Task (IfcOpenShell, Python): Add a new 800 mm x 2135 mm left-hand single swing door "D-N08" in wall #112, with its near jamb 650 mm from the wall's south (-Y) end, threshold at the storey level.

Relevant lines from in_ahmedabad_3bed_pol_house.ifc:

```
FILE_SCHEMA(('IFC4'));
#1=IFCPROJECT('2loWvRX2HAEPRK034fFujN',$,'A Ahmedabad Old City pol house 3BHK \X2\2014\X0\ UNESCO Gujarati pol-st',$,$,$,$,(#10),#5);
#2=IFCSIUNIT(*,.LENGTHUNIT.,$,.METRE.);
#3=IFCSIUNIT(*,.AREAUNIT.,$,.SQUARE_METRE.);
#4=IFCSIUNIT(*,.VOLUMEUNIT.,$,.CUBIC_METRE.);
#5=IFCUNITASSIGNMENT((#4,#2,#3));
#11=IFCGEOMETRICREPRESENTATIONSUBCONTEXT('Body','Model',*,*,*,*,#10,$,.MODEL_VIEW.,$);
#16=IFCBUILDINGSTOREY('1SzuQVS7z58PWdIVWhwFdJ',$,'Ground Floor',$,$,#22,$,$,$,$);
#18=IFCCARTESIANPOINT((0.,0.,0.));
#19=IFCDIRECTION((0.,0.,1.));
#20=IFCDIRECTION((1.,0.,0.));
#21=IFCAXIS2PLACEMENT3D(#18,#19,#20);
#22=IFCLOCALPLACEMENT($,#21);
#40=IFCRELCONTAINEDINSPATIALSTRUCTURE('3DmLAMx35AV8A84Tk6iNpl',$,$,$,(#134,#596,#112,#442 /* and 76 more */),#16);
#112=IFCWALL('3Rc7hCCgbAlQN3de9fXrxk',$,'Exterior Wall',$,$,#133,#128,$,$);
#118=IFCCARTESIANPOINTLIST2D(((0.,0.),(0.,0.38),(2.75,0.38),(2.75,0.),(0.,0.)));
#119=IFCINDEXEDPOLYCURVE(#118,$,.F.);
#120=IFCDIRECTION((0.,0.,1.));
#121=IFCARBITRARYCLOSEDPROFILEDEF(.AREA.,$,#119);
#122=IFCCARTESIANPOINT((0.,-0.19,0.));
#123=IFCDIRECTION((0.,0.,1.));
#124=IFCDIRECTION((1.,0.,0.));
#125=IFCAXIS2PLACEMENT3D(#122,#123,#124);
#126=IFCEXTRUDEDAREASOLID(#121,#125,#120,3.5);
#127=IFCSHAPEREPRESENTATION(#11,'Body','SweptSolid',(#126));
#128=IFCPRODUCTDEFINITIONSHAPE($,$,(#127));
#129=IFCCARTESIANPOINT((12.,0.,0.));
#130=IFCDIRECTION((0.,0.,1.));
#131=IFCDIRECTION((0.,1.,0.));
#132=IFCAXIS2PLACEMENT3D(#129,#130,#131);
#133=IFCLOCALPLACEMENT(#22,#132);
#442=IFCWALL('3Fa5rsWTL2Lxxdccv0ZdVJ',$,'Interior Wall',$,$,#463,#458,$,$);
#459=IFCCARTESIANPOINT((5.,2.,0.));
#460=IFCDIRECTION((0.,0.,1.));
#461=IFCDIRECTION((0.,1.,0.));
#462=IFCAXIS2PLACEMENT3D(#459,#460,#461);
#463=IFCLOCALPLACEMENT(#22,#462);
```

```python
import numpy as np
import ifcopenshell
import ifcopenshell.api.feature
import ifcopenshell.api.geometry
import ifcopenshell.api.root
import ifcopenshell.api.spatial
import ifcopenshell.geom
import ifcopenshell.util.element
import ifcopenshell.util.placement
import ifcopenshell.util.representation
import ifcopenshell.util.shape
import ifcopenshell.util.unit

model = ifcopenshell.open("in_ahmedabad_3bed_pol_house.ifc")
unit_scale = ifcopenshell.util.unit.calculate_unit_scale(model)
settings = ifcopenshell.geom.settings()


def volume(element):
    """Net volume in cubic metres, openings subtracted."""
    shape = ifcopenshell.geom.create_shape(settings, element)
    return ifcopenshell.util.shape.get_volume(shape.geometry)


wall = model.by_id(112)
storey = ifcopenshell.util.element.get_container(wall, ifc_class="IfcBuildingStorey")
context = ifcopenshell.util.representation.get_context(model, "Model", "Body", "MODEL_VIEW")
before = volume(wall)

width, height, from_end, sill = 0.8, 2.135, 0.65, 0.0  # metres

# The wall runs along its own X axis, and the end named is its -X end.
wall_shape = ifcopenshell.geom.create_shape(settings, wall)
x, y, z = ifcopenshell.util.shape.get_vertices(wall_shape.geometry).T
start = x.min() + from_end
face, thickness = float(y.min()), float(y.max() - y.min())
wall_matrix = ifcopenshell.util.placement.get_local_placement(wall.ObjectPlacement)
level = ifcopenshell.util.placement.get_local_placement(storey.ObjectPlacement)[2, 3]


def in_wall(x, y):
    """Placement at x, y metres in the wall's axes, at sill height."""
    matrix = wall_matrix.copy()
    matrix[:, 3] = wall_matrix @ np.array([x / unit_scale, y / unit_scale, 0.0, 1.0])
    matrix[2, 3] = level + sill / unit_scale
    return matrix


# Opening: a box that overshoots both wall faces by 50 mm.
opening = ifcopenshell.api.root.create_entity(model, ifc_class="IfcOpeningElement", predefined_type="OPENING")
box = ifcopenshell.api.geometry.add_wall_representation(
    model, context=context, length=width, height=height, thickness=thickness + 0.1
)
ifcopenshell.api.geometry.assign_representation(model, product=opening, representation=box)
ifcopenshell.api.geometry.edit_object_placement(model, product=opening, matrix=in_wall(start, face - 0.05), is_si=False)
ifcopenshell.api.feature.add_feature(model, feature=opening, element=wall)

door = ifcopenshell.api.root.create_entity(model, ifc_class="IfcDoor", name="D-N08", predefined_type="DOOR")
door.OverallWidth, door.OverallHeight = width / unit_scale, height / unit_scale
door.OperationType = "SINGLE_SWING_LEFT"
body = ifcopenshell.api.geometry.add_door_representation(
    model,
    context=context,
    overall_width=door.OverallWidth,
    overall_height=door.OverallHeight,
    operation_type="SINGLE_SWING_LEFT",
    lining_properties={"LiningDepth": thickness / unit_scale, "ThresholdDepth": thickness / unit_scale},
)
ifcopenshell.api.geometry.assign_representation(model, product=door, representation=body)
ifcopenshell.api.spatial.assign_container(model, products=[door], relating_structure=storey)
ifcopenshell.api.feature.add_filling(model, opening=opening, element=door)

# The lining spans the wall, so the door starts at the wall face.
ifcopenshell.api.geometry.edit_object_placement(model, product=door, matrix=in_wall(start, face), is_si=False)

after = volume(wall)

print(f"wall volume {before:.3f} -> {after:.3f} m3")

model.write("in_ahmedabad_3bed_pol_house-out.ifc")
```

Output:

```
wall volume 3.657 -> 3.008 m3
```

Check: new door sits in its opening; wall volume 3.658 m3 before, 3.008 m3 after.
